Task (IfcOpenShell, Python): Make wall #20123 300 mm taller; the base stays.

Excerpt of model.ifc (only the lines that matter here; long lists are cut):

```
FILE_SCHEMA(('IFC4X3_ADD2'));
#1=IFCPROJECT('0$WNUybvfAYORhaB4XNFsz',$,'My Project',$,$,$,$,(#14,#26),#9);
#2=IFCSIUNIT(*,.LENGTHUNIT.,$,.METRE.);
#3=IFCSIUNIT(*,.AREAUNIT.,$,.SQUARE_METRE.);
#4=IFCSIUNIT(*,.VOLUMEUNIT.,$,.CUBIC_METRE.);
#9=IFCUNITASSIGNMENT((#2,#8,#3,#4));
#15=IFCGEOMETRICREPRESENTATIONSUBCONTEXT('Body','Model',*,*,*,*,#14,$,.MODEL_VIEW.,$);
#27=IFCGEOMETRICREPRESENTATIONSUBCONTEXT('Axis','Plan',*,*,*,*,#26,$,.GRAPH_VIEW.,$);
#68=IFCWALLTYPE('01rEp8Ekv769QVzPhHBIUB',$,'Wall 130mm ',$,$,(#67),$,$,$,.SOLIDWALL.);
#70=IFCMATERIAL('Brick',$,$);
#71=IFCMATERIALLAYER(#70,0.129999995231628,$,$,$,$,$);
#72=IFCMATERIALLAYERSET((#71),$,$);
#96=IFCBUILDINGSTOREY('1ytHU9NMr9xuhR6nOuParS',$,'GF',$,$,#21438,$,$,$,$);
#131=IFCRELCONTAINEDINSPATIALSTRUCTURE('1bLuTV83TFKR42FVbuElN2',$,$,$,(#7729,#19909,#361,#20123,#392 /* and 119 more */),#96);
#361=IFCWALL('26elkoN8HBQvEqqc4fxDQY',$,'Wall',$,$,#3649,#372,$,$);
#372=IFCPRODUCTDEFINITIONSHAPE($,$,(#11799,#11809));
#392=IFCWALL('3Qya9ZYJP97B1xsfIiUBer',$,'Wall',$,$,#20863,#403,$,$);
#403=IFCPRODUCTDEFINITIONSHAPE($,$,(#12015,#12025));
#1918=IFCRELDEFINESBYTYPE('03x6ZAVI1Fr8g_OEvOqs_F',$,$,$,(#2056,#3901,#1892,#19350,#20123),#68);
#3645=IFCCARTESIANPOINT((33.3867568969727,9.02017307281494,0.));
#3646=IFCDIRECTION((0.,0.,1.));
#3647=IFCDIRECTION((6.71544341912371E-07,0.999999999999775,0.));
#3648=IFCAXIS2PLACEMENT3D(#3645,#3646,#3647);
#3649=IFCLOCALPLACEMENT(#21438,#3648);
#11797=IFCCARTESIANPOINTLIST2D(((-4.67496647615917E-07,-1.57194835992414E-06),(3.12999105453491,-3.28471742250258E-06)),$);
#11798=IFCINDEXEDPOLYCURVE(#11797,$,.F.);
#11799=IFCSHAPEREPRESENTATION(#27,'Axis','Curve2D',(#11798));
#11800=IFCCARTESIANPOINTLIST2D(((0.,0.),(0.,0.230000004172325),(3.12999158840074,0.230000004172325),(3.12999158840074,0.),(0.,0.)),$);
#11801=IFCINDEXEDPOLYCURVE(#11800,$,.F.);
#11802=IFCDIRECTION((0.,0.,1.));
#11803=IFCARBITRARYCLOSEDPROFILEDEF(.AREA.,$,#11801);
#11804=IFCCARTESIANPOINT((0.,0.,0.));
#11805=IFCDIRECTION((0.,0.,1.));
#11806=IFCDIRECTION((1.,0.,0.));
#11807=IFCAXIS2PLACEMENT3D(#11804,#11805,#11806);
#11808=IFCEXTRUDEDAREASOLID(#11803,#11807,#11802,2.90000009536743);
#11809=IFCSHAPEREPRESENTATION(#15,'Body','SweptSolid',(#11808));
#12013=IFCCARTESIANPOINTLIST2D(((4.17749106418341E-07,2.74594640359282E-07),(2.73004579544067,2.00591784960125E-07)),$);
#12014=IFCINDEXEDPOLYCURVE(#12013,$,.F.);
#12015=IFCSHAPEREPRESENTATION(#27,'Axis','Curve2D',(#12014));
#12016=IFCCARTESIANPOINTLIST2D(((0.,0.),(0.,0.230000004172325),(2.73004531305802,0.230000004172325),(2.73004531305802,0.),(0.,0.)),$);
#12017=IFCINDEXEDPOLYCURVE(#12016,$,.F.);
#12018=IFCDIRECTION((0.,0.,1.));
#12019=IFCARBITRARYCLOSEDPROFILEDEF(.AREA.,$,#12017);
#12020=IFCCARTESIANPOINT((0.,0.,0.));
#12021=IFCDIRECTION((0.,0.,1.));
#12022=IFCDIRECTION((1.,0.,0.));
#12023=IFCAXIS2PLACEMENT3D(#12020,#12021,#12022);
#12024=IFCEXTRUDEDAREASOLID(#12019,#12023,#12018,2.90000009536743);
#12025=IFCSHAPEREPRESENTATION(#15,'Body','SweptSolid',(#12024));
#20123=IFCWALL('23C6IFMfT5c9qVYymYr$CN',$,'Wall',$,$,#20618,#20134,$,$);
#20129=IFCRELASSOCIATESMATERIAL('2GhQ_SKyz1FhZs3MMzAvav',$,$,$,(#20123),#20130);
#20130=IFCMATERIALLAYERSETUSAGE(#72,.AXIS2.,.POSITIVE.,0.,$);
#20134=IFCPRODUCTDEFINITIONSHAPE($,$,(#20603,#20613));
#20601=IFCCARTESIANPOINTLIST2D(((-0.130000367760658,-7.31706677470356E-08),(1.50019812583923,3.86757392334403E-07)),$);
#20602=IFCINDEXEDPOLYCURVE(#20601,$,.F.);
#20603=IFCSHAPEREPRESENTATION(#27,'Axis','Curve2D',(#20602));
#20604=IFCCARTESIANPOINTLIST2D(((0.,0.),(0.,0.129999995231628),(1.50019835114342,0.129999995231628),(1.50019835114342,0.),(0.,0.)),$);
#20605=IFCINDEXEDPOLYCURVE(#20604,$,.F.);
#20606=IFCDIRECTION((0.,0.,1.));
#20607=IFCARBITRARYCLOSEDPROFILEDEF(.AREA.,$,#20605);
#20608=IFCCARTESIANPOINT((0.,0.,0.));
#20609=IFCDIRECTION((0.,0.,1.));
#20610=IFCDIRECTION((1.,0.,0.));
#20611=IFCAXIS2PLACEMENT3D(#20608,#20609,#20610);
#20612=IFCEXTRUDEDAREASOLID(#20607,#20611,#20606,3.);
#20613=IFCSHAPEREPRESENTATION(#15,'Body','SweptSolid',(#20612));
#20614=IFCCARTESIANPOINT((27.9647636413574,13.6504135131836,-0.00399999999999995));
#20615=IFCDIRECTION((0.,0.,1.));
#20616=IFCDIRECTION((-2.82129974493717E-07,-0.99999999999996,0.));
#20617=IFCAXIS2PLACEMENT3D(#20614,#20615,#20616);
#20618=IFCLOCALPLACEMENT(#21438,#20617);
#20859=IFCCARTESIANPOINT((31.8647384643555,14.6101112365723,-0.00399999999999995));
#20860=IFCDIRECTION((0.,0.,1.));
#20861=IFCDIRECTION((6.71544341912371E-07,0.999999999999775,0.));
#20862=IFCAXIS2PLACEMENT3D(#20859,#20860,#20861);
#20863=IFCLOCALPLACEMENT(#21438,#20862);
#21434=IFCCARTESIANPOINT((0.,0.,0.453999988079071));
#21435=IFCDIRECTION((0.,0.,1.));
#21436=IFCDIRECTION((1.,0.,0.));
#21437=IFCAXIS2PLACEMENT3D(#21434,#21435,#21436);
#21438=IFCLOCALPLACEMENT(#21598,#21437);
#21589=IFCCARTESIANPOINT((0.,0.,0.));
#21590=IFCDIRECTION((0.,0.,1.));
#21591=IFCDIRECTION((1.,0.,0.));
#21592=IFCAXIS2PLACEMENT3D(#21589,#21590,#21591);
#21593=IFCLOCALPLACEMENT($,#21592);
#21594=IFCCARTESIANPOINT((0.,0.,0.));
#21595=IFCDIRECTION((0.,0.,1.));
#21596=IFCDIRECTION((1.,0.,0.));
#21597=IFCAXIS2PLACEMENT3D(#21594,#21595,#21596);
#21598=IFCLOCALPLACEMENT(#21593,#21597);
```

```python
import ifcopenshell
import ifcopenshell.geom
import ifcopenshell.util.representation
import ifcopenshell.util.shape
import ifcopenshell.util.unit

model = ifcopenshell.open("model.ifc")
unit_scale = ifcopenshell.util.unit.calculate_unit_scale(model)
settings = ifcopenshell.geom.settings()


def volume(element):
    """Net volume in cubic metres, openings subtracted."""
    shape = ifcopenshell.geom.create_shape(settings, element)
    return ifcopenshell.util.shape.get_volume(shape.geometry)


wall = model.by_guid("23C6IFMfT5c9qVYymYr$CN")
before = volume(wall)

body = ifcopenshell.util.representation.get_representation(wall, "Model", "Body")
solid = body.Items[0]
old_height = solid.Depth
solid.Depth += 0.3 / unit_scale
after = volume(wall)

print(f"height {old_height:g} -> {solid.Depth:g}, volume {before:.3f} -> {after:.3f} m3")

model.write("model-out.ifc")
```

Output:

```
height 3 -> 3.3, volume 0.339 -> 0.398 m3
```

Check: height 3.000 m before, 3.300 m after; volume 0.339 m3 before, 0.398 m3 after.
